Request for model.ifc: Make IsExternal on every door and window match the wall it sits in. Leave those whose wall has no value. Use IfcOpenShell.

First a look at what the model holds.

```python
import ifcopenshell
import ifcopenshell.util.element

model = ifcopenshell.open("model.ifc")
print(model.schema)
seen = {}
for e in model.by_type("IfcDoor") + model.by_type("IfcWindow"):
    if not e.FillsVoids:
        continue
    host = e.FillsVoids[0].RelatingOpeningElement.VoidsElements[0].RelatingBuildingElement
    own = ifcopenshell.util.element.get_pset(e, f"Pset_{e.is_a()[3:].removesuffix('StandardCase')}Common", "IsExternal")
    wall = ifcopenshell.util.element.get_pset(host, "Pset_WallCommon", "IsExternal")
    seen[e.is_a(), own, wall] = seen.get((e.is_a(), own, wall), 0) + 1
for (cls, own, wall), count in sorted(seen.items(), key=str):
    print(count, cls, "IsExternal:", own, "| host wall:", wall)
```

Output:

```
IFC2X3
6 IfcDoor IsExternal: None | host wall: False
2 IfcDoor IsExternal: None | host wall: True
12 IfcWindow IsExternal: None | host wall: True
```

```python
import ifcopenshell
import ifcopenshell.api.pset
import ifcopenshell.util.element

model = ifcopenshell.open("model.ifc")

count = 0
for ifc_class, pset_name in (("IfcDoor", "Pset_DoorCommon"), ("IfcWindow", "Pset_WindowCommon")):
    for e in model.by_type(ifc_class):
        if not e.FillsVoids:
            continue
        host = e.FillsVoids[0].RelatingOpeningElement.VoidsElements[0].RelatingBuildingElement
        external = ifcopenshell.util.element.get_pset(host, "Pset_WallCommon", "IsExternal")
        if external is None or ifcopenshell.util.element.get_pset(e, pset_name, "IsExternal") == external:
            continue
        pset = ifcopenshell.api.pset.add_pset(model, product=e, name=pset_name)
        ifcopenshell.api.pset.edit_pset(model, pset=pset, properties={"IsExternal": external})
        count += 1

print(count, "updated")

model.write("model_updated.ifc")
```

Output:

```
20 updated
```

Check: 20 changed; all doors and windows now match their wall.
